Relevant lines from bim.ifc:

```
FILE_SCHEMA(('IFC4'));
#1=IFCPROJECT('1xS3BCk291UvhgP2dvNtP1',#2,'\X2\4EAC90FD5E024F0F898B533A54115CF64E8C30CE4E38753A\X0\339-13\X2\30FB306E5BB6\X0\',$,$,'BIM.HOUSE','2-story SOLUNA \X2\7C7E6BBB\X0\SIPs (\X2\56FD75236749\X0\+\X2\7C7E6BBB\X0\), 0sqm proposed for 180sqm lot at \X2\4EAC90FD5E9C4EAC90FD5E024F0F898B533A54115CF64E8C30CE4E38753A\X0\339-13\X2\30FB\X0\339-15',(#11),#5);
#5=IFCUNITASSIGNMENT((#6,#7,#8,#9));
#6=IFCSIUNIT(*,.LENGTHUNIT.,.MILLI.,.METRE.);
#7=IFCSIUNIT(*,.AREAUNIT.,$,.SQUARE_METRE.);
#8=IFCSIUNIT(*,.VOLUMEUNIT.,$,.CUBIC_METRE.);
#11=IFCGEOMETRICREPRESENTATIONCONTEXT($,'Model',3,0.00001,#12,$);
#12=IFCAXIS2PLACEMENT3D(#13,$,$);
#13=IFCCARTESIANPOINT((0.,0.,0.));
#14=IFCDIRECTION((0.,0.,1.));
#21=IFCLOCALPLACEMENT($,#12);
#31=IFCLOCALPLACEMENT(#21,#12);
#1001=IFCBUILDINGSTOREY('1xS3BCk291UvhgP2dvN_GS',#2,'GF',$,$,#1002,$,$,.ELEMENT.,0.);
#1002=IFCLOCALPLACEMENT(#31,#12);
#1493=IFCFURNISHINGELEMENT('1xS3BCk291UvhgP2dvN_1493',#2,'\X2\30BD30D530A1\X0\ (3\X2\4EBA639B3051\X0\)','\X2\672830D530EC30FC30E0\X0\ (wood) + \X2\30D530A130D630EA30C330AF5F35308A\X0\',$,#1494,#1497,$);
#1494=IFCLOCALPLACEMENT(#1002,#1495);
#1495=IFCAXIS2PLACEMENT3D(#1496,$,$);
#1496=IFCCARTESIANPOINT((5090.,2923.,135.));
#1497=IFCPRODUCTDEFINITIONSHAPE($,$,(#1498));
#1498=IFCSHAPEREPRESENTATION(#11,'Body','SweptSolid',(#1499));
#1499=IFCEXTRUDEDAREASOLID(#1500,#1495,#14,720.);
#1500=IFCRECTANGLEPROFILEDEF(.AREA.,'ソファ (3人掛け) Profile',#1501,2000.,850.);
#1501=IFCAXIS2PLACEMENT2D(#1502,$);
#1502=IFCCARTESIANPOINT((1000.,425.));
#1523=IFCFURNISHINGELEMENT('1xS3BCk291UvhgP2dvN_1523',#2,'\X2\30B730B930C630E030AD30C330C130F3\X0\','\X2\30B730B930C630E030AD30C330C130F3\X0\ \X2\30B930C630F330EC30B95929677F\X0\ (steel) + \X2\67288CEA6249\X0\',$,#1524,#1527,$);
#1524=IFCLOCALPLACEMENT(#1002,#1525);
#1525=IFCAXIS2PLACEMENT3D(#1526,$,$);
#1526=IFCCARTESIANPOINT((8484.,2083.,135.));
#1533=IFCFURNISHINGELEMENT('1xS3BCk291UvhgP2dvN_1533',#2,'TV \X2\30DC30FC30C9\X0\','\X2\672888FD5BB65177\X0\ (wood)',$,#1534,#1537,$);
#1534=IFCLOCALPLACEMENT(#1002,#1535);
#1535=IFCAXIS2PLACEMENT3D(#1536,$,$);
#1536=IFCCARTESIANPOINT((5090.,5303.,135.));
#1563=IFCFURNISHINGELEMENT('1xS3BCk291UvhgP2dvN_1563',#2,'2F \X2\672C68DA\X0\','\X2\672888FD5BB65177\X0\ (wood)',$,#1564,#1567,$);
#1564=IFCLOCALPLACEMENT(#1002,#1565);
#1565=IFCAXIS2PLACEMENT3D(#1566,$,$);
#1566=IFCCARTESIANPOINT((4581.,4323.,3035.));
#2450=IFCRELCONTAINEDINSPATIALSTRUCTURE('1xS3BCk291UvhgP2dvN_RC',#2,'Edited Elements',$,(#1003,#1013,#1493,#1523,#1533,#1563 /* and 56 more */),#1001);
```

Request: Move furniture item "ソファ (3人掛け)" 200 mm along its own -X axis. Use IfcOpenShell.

```python
import ifcopenshell
import ifcopenshell.api.geometry
import ifcopenshell.util.placement

model = ifcopenshell.open("bim.ifc")

item = model.by_guid("1xS3BCk291UvhgP2dvN_1493")
matrix = ifcopenshell.util.placement.get_local_placement(item.ObjectPlacement)
matrix[:3, 3] -= matrix[:3, 0] * 200.0
ifcopenshell.api.geometry.edit_object_placement(model, product=item, matrix=matrix, is_si=False)

print(ifcopenshell.util.placement.get_local_placement(item.ObjectPlacement).round(3) + 0.0)

model.write("bim_edited.ifc")
```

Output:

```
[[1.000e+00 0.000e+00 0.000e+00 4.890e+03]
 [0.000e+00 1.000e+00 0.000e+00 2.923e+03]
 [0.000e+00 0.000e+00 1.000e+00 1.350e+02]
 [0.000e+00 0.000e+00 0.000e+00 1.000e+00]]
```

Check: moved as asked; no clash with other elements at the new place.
